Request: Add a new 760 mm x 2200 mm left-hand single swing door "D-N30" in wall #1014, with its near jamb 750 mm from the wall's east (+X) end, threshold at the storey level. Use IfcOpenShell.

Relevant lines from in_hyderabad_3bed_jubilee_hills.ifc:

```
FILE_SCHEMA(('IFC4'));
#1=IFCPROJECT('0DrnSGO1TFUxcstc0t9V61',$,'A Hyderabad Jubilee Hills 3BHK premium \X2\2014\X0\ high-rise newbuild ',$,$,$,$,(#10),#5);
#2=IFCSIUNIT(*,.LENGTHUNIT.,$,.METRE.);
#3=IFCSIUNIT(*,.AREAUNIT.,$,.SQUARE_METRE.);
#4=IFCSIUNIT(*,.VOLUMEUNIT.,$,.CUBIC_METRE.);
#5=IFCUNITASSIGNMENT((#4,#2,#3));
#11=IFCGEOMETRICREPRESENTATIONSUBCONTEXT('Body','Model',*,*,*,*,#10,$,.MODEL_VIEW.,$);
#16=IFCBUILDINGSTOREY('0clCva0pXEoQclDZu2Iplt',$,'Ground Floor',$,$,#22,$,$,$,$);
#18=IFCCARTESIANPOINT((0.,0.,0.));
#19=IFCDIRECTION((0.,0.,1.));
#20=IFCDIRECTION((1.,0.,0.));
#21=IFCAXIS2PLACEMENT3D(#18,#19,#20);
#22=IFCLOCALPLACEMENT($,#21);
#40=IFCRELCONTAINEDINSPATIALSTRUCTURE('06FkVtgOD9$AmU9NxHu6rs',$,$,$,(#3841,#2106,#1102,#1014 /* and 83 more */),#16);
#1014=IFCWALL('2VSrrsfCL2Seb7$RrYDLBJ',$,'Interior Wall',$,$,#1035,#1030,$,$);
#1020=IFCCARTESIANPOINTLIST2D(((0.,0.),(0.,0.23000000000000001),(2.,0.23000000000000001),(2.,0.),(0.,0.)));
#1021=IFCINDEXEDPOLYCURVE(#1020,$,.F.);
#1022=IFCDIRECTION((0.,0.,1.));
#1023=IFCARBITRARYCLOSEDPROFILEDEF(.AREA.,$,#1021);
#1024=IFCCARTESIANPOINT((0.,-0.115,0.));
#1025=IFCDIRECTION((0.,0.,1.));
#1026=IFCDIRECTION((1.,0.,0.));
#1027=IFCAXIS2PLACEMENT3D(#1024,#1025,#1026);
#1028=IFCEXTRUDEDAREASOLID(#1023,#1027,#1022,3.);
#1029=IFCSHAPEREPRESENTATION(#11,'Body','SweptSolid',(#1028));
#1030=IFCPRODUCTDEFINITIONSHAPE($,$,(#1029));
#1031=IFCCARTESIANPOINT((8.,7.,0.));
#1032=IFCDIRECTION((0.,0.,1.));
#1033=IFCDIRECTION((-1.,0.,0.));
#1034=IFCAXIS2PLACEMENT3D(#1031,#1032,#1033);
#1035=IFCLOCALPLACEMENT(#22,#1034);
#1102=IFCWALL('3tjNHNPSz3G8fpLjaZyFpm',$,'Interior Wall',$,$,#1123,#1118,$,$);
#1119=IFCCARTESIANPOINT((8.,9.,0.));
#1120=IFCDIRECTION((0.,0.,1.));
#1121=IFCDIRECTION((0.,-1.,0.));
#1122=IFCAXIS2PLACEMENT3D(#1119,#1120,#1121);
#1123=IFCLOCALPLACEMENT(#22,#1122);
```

```python
import numpy as np
import ifcopenshell
import ifcopenshell.api.feature
import ifcopenshell.api.geometry
import ifcopenshell.api.root
import ifcopenshell.api.spatial
import ifcopenshell.geom
import ifcopenshell.util.element
import ifcopenshell.util.placement
import ifcopenshell.util.representation
import ifcopenshell.util.shape
import ifcopenshell.util.unit

model = ifcopenshell.open("in_hyderabad_3bed_jubilee_hills.ifc")
unit_scale = ifcopenshell.util.unit.calculate_unit_scale(model)
settings = ifcopenshell.geom.settings()


def volume(element):
    """Net volume in cubic metres, openings subtracted."""
    shape = ifcopenshell.geom.create_shape(settings, element)
    return ifcopenshell.util.shape.get_volume(shape.geometry)


wall = model.by_id(1014)
storey = ifcopenshell.util.element.get_container(wall, ifc_class="IfcBuildingStorey")
context = ifcopenshell.util.representation.get_context(model, "Model", "Body", "MODEL_VIEW")
before = volume(wall)

width, height, from_end, sill = 0.76, 2.2, 0.75, 0.0  # metres

# The wall runs along its own X axis, and the end named is its -X end.
wall_shape = ifcopenshell.geom.create_shape(settings, wall)
x, y, z = ifcopenshell.util.shape.get_vertices(wall_shape.geometry).T
start = x.min() + from_end
face, thickness = float(y.min()), float(y.max() - y.min())
wall_matrix = ifcopenshell.util.placement.get_local_placement(wall.ObjectPlacement)
level = ifcopenshell.util.placement.get_local_placement(storey.ObjectPlacement)[2, 3]


def in_wall(x, y):
    """Placement at x, y metres in the wall's axes, at sill height."""
    matrix = wall_matrix.copy()
    matrix[:, 3] = wall_matrix @ np.array([x / unit_scale, y / unit_scale, 0.0, 1.0])
    matrix[2, 3] = level + sill / unit_scale
    return matrix


# Opening: a box that overshoots both wall faces by 50 mm.
opening = ifcopenshell.api.root.create_entity(model, ifc_class="IfcOpeningElement", predefined_type="OPENING")
box = ifcopenshell.api.geometry.add_wall_representation(
    model, context=context, length=width, height=height, thickness=thickness + 0.1
)
ifcopenshell.api.geometry.assign_representation(model, product=opening, representation=box)
ifcopenshell.api.geometry.edit_object_placement(model, product=opening, matrix=in_wall(start, face - 0.05), is_si=False)
ifcopenshell.api.feature.add_feature(model, feature=opening, element=wall)

door = ifcopenshell.api.root.create_entity(model, ifc_class="IfcDoor", name="D-N30", predefined_type="DOOR")
door.OverallWidth, door.OverallHeight = width / unit_scale, height / unit_scale
door.OperationType = "SINGLE_SWING_LEFT"
body = ifcopenshell.api.geometry.add_door_representation(
    model,
    context=context,
    overall_width=door.OverallWidth,
    overall_height=door.OverallHeight,
    operation_type="SINGLE_SWING_LEFT",
    lining_properties={"LiningDepth": thickness / unit_scale, "ThresholdDepth": thickness / unit_scale},
)
ifcopenshell.api.geometry.assign_representation(model, product=door, representation=body)
ifcopenshell.api.spatial.assign_container(model, products=[door], relating_structure=storey)
ifcopenshell.api.feature.add_filling(model, opening=opening, element=door)

# The lining spans the wall, so the door starts at the wall face.
ifcopenshell.api.geometry.edit_object_placement(model, product=door, matrix=in_wall(start, face), is_si=False)

after = volume(wall)

print(f"wall volume {before:.3f} -> {after:.3f} m3")

model.write("in_hyderabad_3bed_jubilee_hills_edited.ifc")
```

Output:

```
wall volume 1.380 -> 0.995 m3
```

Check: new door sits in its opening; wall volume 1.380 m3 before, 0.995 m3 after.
